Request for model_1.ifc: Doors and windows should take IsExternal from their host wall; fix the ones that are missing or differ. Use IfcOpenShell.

First a look at what the model holds.

```python
import ifcopenshell
import ifcopenshell.util.element

model = ifcopenshell.open("model_1.ifc")
print(model.schema)
seen = {}
for e in model.by_type("IfcDoor") + model.by_type("IfcWindow"):
    if not e.FillsVoids:
        continue
    host = e.FillsVoids[0].RelatingOpeningElement.VoidsElements[0].RelatingBuildingElement
    own = ifcopenshell.util.element.get_pset(e, f"Pset_{e.is_a()[3:].removesuffix('StandardCase')}Common", "IsExternal")
    wall = ifcopenshell.util.element.get_pset(host, "Pset_WallCommon", "IsExternal")
    seen[e.is_a(), own, wall] = seen.get((e.is_a(), own, wall), 0) + 1
for (cls, own, wall), count in sorted(seen.items(), key=str):
    print(count, cls, "IsExternal:", own, "| host wall:", wall)
```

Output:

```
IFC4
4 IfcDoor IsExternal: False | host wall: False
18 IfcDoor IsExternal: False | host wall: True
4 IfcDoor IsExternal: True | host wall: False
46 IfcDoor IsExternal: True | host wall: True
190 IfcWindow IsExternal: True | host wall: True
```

```python
import ifcopenshell
import ifcopenshell.api.pset
import ifcopenshell.util.element

model = ifcopenshell.open("model_1.ifc")

count = 0
for ifc_class, pset_name in (("IfcDoor", "Pset_DoorCommon"), ("IfcWindow", "Pset_WindowCommon")):
    for e in model.by_type(ifc_class):
        if not e.FillsVoids:
            continue
        host = e.FillsVoids[0].RelatingOpeningElement.VoidsElements[0].RelatingBuildingElement
        external = ifcopenshell.util.element.get_pset(host, "Pset_WallCommon", "IsExternal")
        if external is None or ifcopenshell.util.element.get_pset(e, pset_name, "IsExternal") == external:
            continue
        pset = ifcopenshell.api.pset.add_pset(model, product=e, name=pset_name)
        ifcopenshell.api.pset.edit_pset(model, pset=pset, properties={"IsExternal": external})
        count += 1

print(count, "updated")

model.write("model_1_edited.ifc")
```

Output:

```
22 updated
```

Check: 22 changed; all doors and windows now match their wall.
